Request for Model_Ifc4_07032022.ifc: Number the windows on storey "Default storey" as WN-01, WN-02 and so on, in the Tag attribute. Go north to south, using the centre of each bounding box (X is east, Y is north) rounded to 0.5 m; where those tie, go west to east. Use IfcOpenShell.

First a look at what the model holds.

```python
import ifcopenshell
import ifcopenshell.util.element
import ifcopenshell.util.placement

model = ifcopenshell.open("Model_Ifc4_07032022.ifc")
print(model.schema)
storey = next(s for s in model.by_type("IfcBuildingStorey") if s.Name == "Default storey")
windows = [e for e in ifcopenshell.util.element.get_decomposition(storey) if e.is_a("IfcWindow")]
for e in sorted(windows, key=lambda e: e.id()):
    origin = ifcopenshell.util.placement.get_local_placement(e.ObjectPlacement)[:3, 3]
    print(e.id(), e.Tag, e.Name, origin.round(2) + 0.0, sep=" | ")
```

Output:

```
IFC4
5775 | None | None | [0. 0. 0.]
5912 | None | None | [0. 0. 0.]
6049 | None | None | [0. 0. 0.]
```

```python
import ifcopenshell
import ifcopenshell.geom
import ifcopenshell.util.element
import ifcopenshell.util.shape

model = ifcopenshell.open("Model_Ifc4_07032022.ifc")
settings = ifcopenshell.geom.settings()
settings.set("use-world-coords", True)


def centre(element):
    shape = ifcopenshell.geom.create_shape(settings, element)
    return ifcopenshell.util.shape.get_bbox_centroid(shape.geometry)


storey = next(s for s in model.by_type("IfcBuildingStorey") if s.Name == "Default storey")
windows = [e for e in ifcopenshell.util.element.get_decomposition(storey) if e.is_a("IfcWindow")]

# Insertion points can sit at a corner or the storey origin, so sort by the geometry (in metres).
centres = {e: centre(e) for e in windows}
windows.sort(key=lambda e: (-round(centres[e][1] / 0.5), centres[e][0]))

for i, e in enumerate(windows, start=1):
    number = f"WN-{i:02d}"
    e.Tag = number
    print(e.id(), number)

model.write("Model_Ifc4_07032022_updated.ifc")
```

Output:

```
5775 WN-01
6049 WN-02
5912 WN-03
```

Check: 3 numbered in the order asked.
